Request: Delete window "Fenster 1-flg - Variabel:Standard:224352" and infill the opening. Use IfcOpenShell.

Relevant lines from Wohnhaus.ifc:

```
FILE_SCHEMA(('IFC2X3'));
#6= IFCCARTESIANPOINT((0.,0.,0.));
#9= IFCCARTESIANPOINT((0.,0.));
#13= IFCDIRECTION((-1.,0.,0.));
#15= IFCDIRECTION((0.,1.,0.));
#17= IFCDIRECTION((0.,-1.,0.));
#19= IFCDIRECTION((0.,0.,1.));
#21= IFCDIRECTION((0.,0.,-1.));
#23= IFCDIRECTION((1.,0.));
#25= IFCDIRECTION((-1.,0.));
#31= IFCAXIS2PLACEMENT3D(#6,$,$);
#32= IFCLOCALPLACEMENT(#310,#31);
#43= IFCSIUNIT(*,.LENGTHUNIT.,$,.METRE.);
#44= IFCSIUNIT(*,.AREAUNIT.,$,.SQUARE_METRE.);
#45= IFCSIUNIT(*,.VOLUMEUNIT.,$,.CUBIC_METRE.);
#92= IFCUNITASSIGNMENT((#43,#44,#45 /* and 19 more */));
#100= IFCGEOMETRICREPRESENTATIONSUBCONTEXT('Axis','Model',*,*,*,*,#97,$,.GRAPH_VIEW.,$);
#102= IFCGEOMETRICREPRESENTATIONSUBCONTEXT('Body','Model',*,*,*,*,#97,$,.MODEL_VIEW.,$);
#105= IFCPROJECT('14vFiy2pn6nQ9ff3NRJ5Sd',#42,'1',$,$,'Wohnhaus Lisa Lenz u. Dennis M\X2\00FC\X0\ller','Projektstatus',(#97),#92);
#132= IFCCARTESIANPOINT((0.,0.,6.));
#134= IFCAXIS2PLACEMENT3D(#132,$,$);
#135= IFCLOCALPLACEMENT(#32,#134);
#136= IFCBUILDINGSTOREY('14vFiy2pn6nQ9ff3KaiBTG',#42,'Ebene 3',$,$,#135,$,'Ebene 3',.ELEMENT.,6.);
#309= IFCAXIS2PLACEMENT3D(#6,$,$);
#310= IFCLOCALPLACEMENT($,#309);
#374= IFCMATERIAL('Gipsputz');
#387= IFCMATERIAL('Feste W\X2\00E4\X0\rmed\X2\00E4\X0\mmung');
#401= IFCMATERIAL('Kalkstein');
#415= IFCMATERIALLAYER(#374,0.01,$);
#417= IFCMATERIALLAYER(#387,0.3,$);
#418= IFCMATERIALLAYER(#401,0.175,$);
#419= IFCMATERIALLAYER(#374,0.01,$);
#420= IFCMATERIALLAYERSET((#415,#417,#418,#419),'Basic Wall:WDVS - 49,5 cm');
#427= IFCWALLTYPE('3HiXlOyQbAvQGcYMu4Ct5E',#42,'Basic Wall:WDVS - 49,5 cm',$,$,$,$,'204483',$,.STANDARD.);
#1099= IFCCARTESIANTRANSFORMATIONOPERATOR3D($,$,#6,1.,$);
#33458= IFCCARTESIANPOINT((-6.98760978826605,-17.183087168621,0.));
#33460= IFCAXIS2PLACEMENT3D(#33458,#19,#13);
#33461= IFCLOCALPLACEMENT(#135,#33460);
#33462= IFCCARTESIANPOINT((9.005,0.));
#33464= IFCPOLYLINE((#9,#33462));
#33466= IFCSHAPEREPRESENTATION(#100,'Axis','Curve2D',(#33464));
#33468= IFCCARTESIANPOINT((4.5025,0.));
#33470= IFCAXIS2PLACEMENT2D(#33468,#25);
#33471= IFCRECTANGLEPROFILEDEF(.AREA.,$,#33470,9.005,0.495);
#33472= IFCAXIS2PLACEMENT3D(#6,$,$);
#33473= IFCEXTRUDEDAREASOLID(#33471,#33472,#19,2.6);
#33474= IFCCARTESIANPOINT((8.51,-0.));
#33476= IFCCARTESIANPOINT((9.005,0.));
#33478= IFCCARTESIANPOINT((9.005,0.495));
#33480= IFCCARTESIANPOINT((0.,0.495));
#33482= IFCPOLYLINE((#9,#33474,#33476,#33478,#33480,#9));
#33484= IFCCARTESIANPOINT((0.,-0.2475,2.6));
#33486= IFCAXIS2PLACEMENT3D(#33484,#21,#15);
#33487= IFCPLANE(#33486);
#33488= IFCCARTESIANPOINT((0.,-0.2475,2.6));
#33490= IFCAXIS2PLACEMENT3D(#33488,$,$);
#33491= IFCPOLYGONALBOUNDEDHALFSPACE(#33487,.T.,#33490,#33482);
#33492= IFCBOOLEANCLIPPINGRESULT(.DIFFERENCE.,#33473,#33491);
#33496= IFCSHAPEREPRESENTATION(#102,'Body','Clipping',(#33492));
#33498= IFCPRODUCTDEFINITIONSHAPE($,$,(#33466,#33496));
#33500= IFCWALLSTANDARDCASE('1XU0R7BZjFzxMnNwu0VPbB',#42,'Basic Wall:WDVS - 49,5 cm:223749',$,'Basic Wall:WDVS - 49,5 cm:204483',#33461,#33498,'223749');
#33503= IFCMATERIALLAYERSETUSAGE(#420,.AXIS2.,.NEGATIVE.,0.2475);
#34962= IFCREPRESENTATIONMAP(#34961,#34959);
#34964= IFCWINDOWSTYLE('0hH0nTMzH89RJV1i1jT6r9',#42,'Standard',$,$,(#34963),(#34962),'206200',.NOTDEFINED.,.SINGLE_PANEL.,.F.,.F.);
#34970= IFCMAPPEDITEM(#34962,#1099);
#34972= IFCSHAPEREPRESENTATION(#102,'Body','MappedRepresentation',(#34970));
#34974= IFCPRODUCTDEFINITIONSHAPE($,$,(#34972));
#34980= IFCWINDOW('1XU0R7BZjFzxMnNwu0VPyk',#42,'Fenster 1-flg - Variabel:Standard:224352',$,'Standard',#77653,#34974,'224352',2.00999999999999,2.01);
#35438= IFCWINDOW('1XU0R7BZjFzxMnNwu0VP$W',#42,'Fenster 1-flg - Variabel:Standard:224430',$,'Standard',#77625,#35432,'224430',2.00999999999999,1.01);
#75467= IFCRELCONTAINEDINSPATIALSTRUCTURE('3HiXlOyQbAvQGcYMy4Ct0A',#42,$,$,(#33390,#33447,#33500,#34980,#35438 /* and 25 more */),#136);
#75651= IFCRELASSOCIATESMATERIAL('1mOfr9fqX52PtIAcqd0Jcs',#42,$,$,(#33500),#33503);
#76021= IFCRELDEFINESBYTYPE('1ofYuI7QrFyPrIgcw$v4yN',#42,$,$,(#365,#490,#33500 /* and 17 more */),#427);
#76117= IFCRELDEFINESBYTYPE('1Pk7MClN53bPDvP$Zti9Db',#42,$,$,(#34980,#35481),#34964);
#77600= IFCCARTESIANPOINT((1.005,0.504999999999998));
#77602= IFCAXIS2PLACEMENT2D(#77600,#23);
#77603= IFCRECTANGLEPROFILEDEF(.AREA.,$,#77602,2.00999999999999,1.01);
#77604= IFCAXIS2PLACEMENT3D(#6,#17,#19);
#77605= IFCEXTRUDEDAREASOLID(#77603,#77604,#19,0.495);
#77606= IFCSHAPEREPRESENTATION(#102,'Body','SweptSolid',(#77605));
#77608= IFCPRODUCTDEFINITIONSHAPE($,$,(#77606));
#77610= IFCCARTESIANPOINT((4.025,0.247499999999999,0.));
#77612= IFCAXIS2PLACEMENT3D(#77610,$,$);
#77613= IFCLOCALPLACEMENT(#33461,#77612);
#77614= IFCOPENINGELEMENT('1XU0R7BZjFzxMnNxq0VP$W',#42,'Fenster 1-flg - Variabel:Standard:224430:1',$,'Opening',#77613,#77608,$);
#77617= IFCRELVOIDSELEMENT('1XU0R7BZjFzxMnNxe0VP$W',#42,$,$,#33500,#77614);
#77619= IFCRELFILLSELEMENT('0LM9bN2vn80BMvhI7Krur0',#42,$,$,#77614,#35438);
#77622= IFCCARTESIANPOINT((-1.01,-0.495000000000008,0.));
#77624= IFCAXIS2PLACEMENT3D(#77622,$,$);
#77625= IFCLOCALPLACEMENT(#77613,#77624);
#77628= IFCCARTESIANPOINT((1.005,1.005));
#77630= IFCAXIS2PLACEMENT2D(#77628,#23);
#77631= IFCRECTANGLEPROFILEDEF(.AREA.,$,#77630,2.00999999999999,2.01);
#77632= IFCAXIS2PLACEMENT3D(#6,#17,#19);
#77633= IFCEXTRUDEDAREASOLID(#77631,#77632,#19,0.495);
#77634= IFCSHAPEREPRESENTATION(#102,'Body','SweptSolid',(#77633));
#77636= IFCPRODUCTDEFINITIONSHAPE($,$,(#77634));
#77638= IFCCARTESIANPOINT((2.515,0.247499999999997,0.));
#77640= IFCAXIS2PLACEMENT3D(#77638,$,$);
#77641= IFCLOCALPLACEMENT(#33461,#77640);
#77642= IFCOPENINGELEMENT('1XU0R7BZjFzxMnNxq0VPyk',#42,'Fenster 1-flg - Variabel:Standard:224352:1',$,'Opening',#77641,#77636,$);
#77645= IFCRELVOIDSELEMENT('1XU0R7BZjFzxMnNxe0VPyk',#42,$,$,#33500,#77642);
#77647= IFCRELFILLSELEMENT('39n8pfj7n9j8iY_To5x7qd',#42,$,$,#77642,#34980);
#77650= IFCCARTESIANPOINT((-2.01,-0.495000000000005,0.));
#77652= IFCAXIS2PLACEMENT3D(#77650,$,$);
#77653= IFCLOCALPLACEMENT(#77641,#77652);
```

```python
import ifcopenshell
import ifcopenshell.api.feature
import ifcopenshell.api.root
import ifcopenshell.geom
import ifcopenshell.util.shape

model = ifcopenshell.open("Wohnhaus.ifc")
settings = ifcopenshell.geom.settings()


def volume(element):
    """Net volume in cubic metres, openings subtracted."""
    shape = ifcopenshell.geom.create_shape(settings, element)
    return ifcopenshell.util.shape.get_volume(shape.geometry)


window = model.by_guid("1XU0R7BZjFzxMnNwu0VPyk")
opening = window.FillsVoids[0].RelatingOpeningElement
wall = opening.VoidsElements[0].RelatingBuildingElement
before = volume(wall)

ifcopenshell.api.root.remove_product(model, product=window)
ifcopenshell.api.feature.remove_feature(model, feature=opening)

after = volume(wall)

print(f"wall volume {before:.3f} -> {after:.3f} m3")

model.write("Wohnhaus-out.ifc")
```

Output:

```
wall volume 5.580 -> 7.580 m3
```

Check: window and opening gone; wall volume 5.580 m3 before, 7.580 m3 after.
